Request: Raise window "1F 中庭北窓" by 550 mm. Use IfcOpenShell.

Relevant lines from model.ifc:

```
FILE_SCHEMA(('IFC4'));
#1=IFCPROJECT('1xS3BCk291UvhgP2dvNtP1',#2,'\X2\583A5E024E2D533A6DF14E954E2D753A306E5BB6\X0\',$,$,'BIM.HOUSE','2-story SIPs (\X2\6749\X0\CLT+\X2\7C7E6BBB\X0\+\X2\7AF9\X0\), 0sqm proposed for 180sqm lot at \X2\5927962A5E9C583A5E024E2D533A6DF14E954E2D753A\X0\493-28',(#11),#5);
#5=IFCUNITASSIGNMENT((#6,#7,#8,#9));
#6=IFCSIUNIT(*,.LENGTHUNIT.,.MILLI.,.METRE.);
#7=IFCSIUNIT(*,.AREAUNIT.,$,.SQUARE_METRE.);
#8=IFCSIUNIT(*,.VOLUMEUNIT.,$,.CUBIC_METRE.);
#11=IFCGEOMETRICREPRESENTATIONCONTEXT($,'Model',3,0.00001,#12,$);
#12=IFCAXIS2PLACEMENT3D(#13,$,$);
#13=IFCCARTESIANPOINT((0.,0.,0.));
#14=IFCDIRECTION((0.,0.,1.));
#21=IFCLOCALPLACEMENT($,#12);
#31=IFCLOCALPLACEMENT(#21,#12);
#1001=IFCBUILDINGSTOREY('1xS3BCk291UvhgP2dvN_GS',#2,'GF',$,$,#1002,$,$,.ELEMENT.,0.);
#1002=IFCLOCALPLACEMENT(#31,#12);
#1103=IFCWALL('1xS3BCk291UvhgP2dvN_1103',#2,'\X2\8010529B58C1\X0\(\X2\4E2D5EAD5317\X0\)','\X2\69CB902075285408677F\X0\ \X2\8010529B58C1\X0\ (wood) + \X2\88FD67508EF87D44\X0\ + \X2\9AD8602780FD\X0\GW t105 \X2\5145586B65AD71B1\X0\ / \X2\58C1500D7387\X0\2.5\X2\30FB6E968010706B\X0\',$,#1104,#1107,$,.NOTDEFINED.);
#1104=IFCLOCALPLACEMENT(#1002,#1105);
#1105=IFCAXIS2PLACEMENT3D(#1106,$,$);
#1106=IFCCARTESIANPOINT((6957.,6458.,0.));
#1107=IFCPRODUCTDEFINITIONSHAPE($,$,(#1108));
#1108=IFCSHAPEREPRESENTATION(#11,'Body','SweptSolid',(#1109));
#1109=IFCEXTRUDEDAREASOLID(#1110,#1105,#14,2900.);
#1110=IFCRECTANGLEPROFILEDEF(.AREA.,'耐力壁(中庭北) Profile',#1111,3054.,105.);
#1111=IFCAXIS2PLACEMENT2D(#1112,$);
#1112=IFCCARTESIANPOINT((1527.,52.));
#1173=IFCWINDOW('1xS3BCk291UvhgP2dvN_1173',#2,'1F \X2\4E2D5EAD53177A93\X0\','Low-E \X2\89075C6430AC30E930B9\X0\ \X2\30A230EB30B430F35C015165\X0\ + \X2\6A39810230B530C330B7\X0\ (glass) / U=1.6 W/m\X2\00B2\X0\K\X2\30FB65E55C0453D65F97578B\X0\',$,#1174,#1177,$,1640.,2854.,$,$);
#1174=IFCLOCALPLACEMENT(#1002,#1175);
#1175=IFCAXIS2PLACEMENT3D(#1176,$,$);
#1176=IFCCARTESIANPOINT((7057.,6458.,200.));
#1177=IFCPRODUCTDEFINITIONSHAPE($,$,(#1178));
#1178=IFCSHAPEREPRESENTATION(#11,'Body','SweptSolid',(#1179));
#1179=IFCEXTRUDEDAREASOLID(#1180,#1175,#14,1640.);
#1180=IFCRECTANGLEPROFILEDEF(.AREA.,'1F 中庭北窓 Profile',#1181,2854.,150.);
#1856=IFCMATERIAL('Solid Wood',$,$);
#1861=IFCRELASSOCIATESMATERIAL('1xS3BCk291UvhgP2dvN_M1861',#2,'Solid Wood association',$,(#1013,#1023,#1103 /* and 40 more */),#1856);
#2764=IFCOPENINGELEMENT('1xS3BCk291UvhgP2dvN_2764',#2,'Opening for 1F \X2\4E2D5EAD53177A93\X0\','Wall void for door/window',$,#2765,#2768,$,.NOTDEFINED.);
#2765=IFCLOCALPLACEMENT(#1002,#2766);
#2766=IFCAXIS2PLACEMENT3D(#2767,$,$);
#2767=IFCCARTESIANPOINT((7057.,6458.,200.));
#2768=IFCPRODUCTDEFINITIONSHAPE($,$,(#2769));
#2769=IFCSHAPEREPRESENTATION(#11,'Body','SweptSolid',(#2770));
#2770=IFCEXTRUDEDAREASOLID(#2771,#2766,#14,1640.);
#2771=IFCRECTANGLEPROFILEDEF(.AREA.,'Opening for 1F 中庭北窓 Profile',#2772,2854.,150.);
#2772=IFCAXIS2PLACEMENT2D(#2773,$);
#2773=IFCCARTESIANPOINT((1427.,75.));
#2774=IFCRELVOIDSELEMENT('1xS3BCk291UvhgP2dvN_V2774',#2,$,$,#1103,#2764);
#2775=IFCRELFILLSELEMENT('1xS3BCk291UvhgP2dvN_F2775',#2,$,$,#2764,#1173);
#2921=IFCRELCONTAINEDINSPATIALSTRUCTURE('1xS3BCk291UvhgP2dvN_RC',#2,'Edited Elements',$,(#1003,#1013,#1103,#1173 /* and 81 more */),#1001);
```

```python
import numpy as np
import ifcopenshell
import ifcopenshell.api.geometry
import ifcopenshell.util.placement
import ifcopenshell.util.unit

model = ifcopenshell.open("model.ifc")
unit_scale = ifcopenshell.util.unit.calculate_unit_scale(model)

window = model.by_guid("1xS3BCk291UvhgP2dvN_1173")
opening = window.FillsVoids[0].RelatingOpeningElement
dz = 0.55 / unit_scale

shift = np.array([0.0, 0.0, dz])
# The window is not placed relative to its opening, so move both.
for product in (opening, window):
    matrix = ifcopenshell.util.placement.get_local_placement(product.ObjectPlacement)
    matrix[:3, 3] += shift
    ifcopenshell.api.geometry.edit_object_placement(model, product=product, matrix=matrix, is_si=False)

print(f"moved by {dz * unit_scale:+.3f} m")

model.write("model_v2.ifc")
```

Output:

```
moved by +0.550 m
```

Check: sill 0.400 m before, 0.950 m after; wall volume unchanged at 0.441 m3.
